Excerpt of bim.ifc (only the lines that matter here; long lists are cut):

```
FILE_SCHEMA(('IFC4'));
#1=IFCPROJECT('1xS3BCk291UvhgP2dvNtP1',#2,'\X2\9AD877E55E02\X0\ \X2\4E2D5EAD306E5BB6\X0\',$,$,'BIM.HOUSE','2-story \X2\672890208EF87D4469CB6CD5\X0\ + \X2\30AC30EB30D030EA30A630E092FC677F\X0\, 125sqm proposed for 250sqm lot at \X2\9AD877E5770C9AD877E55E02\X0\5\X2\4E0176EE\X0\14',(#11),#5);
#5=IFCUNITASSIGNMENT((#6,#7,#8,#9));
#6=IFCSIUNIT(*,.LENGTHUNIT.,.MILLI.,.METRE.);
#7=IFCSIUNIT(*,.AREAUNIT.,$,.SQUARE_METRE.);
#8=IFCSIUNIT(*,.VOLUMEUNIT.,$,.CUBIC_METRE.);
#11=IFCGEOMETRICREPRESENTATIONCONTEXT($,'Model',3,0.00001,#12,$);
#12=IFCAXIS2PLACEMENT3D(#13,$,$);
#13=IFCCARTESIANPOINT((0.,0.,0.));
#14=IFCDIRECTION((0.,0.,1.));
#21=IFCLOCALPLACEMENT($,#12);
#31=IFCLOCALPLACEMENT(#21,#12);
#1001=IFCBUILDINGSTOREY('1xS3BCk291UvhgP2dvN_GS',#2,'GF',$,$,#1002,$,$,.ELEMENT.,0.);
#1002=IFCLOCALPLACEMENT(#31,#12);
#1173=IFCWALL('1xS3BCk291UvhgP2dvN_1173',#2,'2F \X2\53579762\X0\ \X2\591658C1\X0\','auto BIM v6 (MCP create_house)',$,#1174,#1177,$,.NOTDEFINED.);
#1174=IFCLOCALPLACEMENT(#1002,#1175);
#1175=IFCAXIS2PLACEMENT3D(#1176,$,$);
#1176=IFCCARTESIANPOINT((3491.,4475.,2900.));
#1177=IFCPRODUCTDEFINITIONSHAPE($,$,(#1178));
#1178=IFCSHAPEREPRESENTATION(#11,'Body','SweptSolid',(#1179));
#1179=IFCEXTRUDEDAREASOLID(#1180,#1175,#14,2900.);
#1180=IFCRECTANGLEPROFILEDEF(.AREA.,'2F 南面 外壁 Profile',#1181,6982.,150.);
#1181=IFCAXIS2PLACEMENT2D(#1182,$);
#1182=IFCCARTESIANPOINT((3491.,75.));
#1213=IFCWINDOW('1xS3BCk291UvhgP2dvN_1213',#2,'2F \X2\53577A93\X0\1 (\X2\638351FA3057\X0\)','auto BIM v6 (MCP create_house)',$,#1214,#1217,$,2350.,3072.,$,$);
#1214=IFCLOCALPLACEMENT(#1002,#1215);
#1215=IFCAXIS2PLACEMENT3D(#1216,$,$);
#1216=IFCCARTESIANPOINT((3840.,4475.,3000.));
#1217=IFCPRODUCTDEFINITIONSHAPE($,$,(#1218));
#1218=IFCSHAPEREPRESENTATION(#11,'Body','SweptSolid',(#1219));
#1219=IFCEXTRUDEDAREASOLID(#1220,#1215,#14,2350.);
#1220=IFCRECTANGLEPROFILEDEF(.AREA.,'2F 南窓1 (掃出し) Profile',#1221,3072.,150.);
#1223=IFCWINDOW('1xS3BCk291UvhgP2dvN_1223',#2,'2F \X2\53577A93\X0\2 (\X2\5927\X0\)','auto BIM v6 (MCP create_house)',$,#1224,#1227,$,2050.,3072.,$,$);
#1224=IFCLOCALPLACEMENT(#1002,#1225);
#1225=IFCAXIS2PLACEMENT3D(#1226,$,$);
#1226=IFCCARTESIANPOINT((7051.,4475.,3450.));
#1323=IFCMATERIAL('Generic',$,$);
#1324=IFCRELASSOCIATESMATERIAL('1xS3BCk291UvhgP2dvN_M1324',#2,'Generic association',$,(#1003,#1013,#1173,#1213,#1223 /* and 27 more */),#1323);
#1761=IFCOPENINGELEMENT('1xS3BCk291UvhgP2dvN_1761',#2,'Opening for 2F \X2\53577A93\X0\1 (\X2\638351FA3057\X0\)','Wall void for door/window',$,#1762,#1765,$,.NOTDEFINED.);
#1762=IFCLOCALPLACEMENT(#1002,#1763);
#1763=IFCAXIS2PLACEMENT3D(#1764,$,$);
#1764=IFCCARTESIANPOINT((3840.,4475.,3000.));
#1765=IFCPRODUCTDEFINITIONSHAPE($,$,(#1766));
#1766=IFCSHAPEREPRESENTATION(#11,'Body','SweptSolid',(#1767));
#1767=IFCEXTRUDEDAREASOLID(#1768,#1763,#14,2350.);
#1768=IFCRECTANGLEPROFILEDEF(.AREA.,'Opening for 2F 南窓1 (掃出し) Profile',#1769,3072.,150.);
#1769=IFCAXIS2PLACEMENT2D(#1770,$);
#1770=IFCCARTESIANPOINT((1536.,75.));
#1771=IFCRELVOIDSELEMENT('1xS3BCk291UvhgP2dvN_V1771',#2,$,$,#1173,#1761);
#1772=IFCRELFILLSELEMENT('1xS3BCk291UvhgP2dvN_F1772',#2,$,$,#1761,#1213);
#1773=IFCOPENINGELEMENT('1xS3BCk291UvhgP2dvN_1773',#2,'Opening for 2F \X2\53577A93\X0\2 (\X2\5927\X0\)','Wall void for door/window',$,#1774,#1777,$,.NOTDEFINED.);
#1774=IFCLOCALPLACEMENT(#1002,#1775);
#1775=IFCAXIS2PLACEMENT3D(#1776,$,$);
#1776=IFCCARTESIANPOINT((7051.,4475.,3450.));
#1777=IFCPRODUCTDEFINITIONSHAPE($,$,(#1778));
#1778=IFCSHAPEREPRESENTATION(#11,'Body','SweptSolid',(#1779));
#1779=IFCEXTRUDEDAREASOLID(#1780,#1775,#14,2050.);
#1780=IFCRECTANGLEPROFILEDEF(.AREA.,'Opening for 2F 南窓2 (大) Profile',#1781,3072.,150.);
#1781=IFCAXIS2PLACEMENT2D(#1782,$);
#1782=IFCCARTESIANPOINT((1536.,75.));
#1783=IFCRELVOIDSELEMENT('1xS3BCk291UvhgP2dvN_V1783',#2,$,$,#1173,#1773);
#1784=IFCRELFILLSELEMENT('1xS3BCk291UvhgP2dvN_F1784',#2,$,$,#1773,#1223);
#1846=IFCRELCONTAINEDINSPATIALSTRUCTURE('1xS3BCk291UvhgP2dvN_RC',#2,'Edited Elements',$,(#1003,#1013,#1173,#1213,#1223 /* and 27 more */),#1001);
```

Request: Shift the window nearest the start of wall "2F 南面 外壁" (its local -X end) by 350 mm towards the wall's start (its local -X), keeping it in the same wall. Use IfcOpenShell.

```python
import ifcopenshell
import ifcopenshell.api.geometry
import ifcopenshell.util.placement
import ifcopenshell.util.unit

model = ifcopenshell.open("bim.ifc")
unit_scale = ifcopenshell.util.unit.calculate_unit_scale(model)

window = model.by_guid("1xS3BCk291UvhgP2dvN_1213")
opening = window.FillsVoids[0].RelatingOpeningElement
wall = opening.VoidsElements[0].RelatingBuildingElement

wall_matrix = ifcopenshell.util.placement.get_local_placement(wall.ObjectPlacement)
shift = wall_matrix[:3, 0] * -0.35 / unit_scale
before = ifcopenshell.util.placement.get_local_placement(window.ObjectPlacement)[:3, 3].copy()

# The window is not placed relative to its opening, so move both.
for product in (opening, window):
    matrix = ifcopenshell.util.placement.get_local_placement(product.ObjectPlacement)
    matrix[:3, 3] += shift
    ifcopenshell.api.geometry.edit_object_placement(model, product=product, matrix=matrix, is_si=False)

after = ifcopenshell.util.placement.get_local_placement(window.ObjectPlacement)[:3, 3]
print("window moved by", (after - before).round(3) + 0.0)

model.write("bim_updated.ifc")
```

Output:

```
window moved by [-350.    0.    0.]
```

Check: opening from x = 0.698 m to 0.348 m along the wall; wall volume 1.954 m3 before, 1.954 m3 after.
